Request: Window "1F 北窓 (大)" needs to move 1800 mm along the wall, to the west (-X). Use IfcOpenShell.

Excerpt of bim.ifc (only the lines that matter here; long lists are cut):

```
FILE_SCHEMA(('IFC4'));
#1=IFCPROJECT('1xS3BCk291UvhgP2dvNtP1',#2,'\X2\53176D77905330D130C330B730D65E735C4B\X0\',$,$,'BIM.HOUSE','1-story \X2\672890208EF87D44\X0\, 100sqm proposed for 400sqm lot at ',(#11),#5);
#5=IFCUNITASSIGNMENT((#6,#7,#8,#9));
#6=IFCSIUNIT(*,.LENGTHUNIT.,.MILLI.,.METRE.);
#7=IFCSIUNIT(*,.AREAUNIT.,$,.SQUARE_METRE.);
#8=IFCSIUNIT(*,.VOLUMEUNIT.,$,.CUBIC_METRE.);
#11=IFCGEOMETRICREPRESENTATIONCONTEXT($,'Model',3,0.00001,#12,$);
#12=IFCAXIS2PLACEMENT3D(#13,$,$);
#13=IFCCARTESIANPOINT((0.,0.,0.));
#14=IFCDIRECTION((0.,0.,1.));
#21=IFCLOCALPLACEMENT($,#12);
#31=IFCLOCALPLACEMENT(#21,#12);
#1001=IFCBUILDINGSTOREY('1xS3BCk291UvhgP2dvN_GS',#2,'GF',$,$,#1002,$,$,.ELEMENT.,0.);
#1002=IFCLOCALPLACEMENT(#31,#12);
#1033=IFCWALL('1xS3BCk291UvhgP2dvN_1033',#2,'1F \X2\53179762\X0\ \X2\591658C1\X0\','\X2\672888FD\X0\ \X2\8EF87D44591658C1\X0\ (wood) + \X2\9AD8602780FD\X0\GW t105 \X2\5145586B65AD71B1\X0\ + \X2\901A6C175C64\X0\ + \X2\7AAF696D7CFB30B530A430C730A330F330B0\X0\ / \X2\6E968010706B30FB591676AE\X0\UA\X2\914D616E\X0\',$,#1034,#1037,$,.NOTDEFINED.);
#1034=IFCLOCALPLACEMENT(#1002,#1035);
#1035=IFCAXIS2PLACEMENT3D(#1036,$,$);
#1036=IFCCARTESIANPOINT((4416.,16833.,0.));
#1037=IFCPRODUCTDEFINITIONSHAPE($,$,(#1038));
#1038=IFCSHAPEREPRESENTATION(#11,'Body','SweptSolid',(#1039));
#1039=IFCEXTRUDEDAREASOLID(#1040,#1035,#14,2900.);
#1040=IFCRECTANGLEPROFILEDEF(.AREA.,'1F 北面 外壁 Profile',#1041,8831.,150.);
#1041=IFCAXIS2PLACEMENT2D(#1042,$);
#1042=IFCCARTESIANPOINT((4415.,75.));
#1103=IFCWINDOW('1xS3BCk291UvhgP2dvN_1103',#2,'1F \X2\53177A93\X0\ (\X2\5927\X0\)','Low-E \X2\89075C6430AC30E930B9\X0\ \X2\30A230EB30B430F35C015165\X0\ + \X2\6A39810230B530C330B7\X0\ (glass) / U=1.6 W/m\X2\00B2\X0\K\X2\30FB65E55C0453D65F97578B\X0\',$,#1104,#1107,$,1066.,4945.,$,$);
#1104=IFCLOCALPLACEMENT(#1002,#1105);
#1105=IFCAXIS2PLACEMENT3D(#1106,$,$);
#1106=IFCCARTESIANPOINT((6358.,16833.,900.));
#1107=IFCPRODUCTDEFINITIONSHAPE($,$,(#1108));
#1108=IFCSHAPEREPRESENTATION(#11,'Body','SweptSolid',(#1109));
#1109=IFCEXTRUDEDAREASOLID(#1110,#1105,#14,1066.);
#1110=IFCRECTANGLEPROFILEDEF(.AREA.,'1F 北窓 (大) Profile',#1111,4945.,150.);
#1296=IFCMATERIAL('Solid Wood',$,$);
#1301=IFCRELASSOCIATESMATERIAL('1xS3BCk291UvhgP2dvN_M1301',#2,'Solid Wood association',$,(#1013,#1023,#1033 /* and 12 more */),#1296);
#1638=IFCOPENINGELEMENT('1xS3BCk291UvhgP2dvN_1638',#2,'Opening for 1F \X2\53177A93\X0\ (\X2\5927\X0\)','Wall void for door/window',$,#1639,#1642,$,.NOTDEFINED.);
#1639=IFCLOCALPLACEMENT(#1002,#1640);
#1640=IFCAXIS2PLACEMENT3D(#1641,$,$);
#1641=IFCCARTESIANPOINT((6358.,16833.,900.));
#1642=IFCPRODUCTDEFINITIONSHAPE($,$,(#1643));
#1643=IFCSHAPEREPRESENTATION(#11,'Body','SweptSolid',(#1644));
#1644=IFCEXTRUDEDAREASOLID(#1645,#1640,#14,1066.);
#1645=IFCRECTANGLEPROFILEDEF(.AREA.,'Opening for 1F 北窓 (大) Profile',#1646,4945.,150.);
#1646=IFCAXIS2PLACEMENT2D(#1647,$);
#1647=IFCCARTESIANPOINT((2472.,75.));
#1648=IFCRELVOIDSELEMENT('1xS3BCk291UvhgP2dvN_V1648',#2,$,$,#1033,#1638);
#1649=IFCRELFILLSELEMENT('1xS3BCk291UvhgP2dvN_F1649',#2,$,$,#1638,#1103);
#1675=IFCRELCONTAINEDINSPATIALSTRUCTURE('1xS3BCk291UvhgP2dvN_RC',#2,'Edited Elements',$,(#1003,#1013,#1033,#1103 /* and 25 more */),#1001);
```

```python
import ifcopenshell
import ifcopenshell.api.geometry
import ifcopenshell.util.placement

model = ifcopenshell.open("bim.ifc")

window = model.by_id(1103)
opening = window.FillsVoids[0].RelatingOpeningElement
wall = opening.VoidsElements[0].RelatingBuildingElement

wall_matrix = ifcopenshell.util.placement.get_local_placement(wall.ObjectPlacement)
shift = wall_matrix[:3, 0] * -1800.0
before = ifcopenshell.util.placement.get_local_placement(window.ObjectPlacement)[:3, 3].copy()

# The window is not placed relative to its opening, so move both.
for product in (opening, window):
    matrix = ifcopenshell.util.placement.get_local_placement(product.ObjectPlacement)
    matrix[:3, 3] += shift
    ifcopenshell.api.geometry.edit_object_placement(model, product=product, matrix=matrix, is_si=False)

after = ifcopenshell.util.placement.get_local_placement(window.ObjectPlacement)[:3, 3]
print("window moved by", (after - before).round(3) + 0.0)

model.write("bim_v2.ifc")
```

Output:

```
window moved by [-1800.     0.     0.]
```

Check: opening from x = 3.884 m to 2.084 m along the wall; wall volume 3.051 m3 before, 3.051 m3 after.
